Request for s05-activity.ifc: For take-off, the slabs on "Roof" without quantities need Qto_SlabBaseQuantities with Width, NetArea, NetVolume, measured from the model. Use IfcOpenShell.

First a look at what the model holds.

```python
import ifcopenshell
import ifcopenshell.util.element
import ifcopenshell.util.unit

model = ifcopenshell.open("s05-activity.ifc")
print(model.schema)
for unit_type in ("LENGTHUNIT", "AREAUNIT", "VOLUMEUNIT"):
    print(unit_type, ifcopenshell.util.unit.calculate_unit_scale(model, unit_type))
storey = next(s for s in model.by_type("IfcBuildingStorey") if s.Name == "Roof")
slabs = [e for e in ifcopenshell.util.element.get_decomposition(storey) if e.is_a("IfcSlab")]
for e in sorted(slabs, key=lambda e: e.id()):
    print(e.id(), e.is_a(), e.Name, list(ifcopenshell.util.element.get_psets(e, qtos_only=True)), sep=" | ")
```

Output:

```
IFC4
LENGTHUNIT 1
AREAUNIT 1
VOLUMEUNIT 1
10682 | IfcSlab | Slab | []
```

```python
import ifcopenshell
import ifcopenshell.api.pset
import ifcopenshell.geom
import ifcopenshell.util.element
import ifcopenshell.util.shape
import ifcopenshell.util.unit

model = ifcopenshell.open("s05-activity.ifc")
unit_scale = ifcopenshell.util.unit.calculate_unit_scale(model)
area_scale = ifcopenshell.util.unit.calculate_unit_scale(model, "AREAUNIT")
volume_scale = ifcopenshell.util.unit.calculate_unit_scale(model, "VOLUMEUNIT")
settings = ifcopenshell.geom.settings()

storey = next(s for s in model.by_type("IfcBuildingStorey") if s.Name == "Roof")
slabs = [e for e in ifcopenshell.util.element.get_decomposition(storey) if e.is_a("IfcSlab")]

for e in sorted(slabs, key=lambda e: e.id()):
    if ifcopenshell.util.element.get_psets(e, qtos_only=True, should_inherit=False):
        continue
    # Geometry comes back in metres, in the element's own axes.
    shape = ifcopenshell.geom.create_shape(settings, e)
    values = {
        "Width": ifcopenshell.util.shape.get_z(shape.geometry) / unit_scale,
        "NetArea": ifcopenshell.util.shape.get_footprint_area(shape.geometry) / area_scale,
        "NetVolume": ifcopenshell.util.shape.get_volume(shape.geometry) / volume_scale,
    }
    qto = ifcopenshell.api.pset.add_qto(model, product=e, name="Qto_SlabBaseQuantities")
    ifcopenshell.api.pset.edit_qto(model, qto=qto, properties=values)
    print(e.id(), {k: round(v, 3) for k, v in values.items()})

model.write("s05-activity_edited.ifc")
```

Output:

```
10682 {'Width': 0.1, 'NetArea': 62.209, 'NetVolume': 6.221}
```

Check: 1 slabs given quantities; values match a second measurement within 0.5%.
